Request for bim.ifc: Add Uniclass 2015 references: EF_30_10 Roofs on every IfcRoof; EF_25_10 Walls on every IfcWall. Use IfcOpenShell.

First a look at what the model holds.

```python
import ifcopenshell

model = ifcopenshell.open("bim.ifc")
print(model.schema)
print("classifications:", [c.Name for c in model.by_type("IfcClassification")])
for ifc_class in ("IfcDoor", "IfcRoof", "IfcStair", "IfcWall", "IfcWindow"):
    print(ifc_class, len(model.by_type(ifc_class)))
```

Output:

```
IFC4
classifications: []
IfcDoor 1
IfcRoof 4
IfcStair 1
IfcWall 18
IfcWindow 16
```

```python
import ifcopenshell
import ifcopenshell.api.classification

model = ifcopenshell.open("bim.ifc")

system = ifcopenshell.api.classification.add_classification(model, classification="Uniclass 2015")

codes = {
    "IfcRoof": ("EF_30_10", "Roofs"),
    "IfcWall": ("EF_25_10", "Walls"),
}
for ifc_class, (code, name) in codes.items():
    products = model.by_type(ifc_class)
    ifcopenshell.api.classification.add_reference(
        model, products=products, classification=system, identification=code, name=name
    )
    print(code, len(products))

model.write("bim_rev.ifc")
```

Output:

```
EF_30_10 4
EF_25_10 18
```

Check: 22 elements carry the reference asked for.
